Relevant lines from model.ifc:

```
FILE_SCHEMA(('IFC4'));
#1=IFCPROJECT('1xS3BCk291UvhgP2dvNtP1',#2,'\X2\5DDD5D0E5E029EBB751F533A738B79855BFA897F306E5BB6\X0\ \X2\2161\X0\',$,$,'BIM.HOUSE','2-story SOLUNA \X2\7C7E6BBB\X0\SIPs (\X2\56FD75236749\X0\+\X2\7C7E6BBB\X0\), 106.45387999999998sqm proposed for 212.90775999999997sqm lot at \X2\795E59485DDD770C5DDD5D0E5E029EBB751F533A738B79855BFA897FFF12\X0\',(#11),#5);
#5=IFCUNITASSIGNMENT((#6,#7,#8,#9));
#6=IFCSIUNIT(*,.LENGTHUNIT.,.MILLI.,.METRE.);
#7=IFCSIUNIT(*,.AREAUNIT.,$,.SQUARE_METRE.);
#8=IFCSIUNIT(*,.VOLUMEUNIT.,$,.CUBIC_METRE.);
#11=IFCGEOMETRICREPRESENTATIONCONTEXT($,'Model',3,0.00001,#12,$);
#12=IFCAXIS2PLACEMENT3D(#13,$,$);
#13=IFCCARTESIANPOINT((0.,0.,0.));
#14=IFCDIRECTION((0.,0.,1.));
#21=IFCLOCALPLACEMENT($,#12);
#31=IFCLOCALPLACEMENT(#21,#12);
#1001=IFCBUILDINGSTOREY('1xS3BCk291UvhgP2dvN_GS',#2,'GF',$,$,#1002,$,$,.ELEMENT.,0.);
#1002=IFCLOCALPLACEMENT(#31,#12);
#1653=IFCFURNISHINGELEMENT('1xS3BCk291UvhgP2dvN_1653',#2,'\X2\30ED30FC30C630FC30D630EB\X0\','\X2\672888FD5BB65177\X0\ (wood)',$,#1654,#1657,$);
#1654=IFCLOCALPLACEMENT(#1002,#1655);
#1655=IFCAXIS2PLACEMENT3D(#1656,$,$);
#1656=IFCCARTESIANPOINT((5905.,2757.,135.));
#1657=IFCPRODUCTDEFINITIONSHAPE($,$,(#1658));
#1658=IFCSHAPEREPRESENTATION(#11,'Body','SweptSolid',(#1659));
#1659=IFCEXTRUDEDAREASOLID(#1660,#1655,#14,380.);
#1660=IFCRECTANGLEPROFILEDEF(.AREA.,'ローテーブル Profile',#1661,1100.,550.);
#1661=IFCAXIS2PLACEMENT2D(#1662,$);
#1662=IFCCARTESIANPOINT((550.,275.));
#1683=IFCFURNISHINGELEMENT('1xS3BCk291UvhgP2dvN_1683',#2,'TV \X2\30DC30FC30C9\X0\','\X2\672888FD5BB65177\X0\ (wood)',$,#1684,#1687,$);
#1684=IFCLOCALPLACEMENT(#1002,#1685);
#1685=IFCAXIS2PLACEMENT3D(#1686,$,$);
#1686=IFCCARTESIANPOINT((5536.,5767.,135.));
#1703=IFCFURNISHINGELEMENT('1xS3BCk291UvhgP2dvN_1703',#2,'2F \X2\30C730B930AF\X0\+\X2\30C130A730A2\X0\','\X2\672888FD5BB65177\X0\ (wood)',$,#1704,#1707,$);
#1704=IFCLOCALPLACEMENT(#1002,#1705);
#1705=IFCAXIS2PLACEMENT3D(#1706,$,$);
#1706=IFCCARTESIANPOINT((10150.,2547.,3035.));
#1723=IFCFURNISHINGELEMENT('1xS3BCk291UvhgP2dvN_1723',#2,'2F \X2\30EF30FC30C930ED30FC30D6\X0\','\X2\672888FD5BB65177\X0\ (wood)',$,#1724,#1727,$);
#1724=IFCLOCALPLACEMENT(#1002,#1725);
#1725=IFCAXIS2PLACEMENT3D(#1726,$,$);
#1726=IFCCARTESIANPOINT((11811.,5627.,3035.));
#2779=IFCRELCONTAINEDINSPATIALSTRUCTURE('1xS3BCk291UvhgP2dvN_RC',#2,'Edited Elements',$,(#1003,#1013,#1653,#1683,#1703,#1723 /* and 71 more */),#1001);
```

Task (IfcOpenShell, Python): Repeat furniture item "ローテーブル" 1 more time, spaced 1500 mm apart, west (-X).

```python
import numpy as np
import ifcopenshell
import ifcopenshell.api.geometry
import ifcopenshell.api.root
import ifcopenshell.util.element
import ifcopenshell.util.placement
import ifcopenshell.util.unit

model = ifcopenshell.open("model.ifc")
unit_scale = ifcopenshell.util.unit.calculate_unit_scale(model)


def reuse_history(source, copy):
    """copy_class also copies each property set's owner history, people and application; keep the originals."""
    for rel in copy.IsDefinedBy:
        if rel.is_a("IfcRelDefinesByProperties") and (history := rel.RelatingPropertyDefinition.OwnerHistory):
            rel.RelatingPropertyDefinition.OwnerHistory = source.OwnerHistory
            ifcopenshell.util.element.remove_deep2(model, history)


source = model.by_id(1653)
base = ifcopenshell.util.placement.get_local_placement(source.ObjectPlacement)
step = np.array([-1.0, 0.0, 0.0]) * 1.5 / unit_scale

for i in range(1, 2):
    copy = ifcopenshell.api.root.copy_class(model, product=source)
    copy.Representation = ifcopenshell.util.element.copy_deep(
        model, source.Representation, exclude=["IfcGeometricRepresentationContext", "IfcRepresentationMap"]
    )
    reuse_history(source, copy)
    matrix = base.copy()
    matrix[:3, 3] += i * step
    print("added at", matrix[:3, 3].round(3) + 0.0)
    ifcopenshell.api.geometry.edit_object_placement(model, product=copy, matrix=matrix, is_si=False)

model.write("model-out.ifc")
```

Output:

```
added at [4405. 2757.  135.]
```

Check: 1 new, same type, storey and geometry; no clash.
